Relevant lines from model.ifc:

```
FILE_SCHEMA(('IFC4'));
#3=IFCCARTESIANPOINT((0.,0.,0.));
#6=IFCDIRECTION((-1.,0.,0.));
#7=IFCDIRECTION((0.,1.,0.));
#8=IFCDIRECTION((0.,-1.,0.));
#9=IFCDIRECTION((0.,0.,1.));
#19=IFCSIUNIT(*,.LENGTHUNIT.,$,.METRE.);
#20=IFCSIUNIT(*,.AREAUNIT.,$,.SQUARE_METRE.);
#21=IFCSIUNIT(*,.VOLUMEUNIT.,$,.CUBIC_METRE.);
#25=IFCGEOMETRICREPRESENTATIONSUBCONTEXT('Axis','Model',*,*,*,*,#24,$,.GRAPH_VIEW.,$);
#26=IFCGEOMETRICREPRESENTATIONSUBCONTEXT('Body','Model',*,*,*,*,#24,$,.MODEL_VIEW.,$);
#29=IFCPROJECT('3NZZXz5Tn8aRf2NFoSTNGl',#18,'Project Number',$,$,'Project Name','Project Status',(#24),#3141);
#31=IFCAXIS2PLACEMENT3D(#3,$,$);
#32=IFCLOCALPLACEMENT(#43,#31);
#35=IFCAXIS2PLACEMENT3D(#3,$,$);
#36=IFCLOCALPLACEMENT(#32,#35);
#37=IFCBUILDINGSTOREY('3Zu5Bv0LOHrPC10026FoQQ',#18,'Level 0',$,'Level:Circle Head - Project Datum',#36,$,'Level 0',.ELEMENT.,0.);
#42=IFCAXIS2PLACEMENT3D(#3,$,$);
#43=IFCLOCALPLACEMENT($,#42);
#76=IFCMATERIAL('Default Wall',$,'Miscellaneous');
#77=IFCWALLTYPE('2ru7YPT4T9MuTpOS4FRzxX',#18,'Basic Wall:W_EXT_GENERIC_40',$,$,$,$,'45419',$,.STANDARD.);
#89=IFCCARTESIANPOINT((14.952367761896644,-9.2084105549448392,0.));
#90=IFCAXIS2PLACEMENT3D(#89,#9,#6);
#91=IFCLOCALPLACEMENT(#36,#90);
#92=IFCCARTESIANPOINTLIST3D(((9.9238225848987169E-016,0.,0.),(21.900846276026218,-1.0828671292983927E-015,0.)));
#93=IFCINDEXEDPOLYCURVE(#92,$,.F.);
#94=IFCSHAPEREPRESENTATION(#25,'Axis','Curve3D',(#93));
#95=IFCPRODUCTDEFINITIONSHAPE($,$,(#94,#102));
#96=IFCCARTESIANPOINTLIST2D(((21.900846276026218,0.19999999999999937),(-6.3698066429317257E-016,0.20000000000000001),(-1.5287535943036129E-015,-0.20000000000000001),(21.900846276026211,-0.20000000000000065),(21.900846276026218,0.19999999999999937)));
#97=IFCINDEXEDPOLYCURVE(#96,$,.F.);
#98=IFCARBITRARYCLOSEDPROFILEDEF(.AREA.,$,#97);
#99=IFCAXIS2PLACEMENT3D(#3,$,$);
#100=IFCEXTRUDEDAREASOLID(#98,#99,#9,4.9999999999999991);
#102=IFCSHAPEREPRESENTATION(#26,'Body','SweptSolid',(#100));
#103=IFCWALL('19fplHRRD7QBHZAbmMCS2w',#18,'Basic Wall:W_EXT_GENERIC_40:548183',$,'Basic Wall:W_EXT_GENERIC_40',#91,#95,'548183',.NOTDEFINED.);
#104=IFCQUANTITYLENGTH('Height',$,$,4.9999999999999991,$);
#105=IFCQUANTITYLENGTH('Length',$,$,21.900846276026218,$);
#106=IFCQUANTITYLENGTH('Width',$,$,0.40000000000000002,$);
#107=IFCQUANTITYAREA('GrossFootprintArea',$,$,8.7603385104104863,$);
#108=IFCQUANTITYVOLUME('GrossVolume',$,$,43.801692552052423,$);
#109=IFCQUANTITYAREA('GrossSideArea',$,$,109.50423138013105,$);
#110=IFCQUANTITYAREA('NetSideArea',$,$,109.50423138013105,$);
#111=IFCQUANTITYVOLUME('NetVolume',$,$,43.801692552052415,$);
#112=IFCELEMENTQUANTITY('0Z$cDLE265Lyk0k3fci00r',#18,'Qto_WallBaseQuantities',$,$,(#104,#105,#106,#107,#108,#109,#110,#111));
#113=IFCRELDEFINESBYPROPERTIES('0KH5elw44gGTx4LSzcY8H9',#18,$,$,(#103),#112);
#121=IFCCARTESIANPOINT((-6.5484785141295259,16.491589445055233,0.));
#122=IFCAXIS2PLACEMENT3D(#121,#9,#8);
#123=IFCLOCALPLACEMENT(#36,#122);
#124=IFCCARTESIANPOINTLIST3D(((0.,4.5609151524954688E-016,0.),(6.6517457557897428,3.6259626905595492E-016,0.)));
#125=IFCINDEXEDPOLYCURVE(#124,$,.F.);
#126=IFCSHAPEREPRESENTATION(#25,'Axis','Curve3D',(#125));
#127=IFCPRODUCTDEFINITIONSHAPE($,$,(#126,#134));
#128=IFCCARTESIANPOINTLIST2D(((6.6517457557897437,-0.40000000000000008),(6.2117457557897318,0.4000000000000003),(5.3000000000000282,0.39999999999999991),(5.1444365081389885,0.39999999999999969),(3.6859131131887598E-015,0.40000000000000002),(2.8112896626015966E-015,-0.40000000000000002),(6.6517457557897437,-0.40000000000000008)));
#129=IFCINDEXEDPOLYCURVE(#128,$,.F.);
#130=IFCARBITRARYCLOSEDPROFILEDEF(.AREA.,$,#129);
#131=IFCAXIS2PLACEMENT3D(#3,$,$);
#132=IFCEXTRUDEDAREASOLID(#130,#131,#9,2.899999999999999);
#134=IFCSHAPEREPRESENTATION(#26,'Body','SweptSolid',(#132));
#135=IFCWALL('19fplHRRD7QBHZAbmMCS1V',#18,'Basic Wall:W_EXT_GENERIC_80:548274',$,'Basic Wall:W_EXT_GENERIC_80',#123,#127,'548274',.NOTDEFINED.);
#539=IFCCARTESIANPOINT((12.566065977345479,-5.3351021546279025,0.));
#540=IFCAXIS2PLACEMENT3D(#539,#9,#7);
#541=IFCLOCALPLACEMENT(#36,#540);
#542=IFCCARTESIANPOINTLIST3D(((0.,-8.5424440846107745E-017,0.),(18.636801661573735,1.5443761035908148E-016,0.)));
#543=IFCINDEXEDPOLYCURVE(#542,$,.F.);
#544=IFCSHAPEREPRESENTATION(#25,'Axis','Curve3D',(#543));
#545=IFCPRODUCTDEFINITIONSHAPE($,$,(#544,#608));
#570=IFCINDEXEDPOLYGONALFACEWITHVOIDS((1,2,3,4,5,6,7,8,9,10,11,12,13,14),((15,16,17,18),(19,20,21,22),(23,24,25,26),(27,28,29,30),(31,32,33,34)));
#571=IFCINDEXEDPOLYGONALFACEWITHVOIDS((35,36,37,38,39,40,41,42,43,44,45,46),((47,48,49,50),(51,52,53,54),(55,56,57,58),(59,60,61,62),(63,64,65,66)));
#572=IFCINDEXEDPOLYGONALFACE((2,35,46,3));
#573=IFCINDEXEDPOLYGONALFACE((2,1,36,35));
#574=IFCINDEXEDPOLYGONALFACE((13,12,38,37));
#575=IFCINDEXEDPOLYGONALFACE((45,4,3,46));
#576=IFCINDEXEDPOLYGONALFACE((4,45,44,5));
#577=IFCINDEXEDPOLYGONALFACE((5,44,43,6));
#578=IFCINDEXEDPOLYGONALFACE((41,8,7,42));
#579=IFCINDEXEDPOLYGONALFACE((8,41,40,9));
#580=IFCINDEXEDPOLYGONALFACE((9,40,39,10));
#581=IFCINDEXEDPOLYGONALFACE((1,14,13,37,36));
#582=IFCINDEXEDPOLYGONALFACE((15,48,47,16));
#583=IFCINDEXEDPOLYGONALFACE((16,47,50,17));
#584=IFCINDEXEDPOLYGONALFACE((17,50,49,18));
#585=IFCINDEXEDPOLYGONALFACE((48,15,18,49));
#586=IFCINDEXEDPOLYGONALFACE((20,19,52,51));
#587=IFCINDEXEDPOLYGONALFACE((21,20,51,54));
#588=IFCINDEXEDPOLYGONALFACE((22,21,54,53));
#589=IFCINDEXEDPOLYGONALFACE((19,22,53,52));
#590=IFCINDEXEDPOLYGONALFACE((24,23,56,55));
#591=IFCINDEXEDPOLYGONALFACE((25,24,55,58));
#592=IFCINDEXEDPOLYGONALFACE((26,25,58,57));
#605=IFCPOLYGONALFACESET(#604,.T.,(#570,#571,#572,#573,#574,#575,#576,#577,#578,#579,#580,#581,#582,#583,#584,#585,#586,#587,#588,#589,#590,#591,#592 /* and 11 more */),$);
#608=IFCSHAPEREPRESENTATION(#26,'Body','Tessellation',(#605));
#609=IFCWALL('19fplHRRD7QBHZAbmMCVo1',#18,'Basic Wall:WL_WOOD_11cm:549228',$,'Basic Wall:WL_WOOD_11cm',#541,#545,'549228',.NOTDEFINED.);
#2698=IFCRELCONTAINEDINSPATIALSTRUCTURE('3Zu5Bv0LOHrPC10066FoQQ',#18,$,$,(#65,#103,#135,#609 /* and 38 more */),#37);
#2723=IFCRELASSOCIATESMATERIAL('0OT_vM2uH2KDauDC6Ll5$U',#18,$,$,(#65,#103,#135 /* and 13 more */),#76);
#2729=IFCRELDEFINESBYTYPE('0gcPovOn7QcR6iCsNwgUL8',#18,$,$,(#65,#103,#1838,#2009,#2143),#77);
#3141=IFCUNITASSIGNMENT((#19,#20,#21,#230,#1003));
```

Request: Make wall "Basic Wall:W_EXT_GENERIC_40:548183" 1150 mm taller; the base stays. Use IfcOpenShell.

```python
import ifcopenshell
import ifcopenshell.api.pset
import ifcopenshell.geom
import ifcopenshell.util.element
import ifcopenshell.util.representation
import ifcopenshell.util.shape
import ifcopenshell.util.unit

model = ifcopenshell.open("model.ifc")
unit_scale = ifcopenshell.util.unit.calculate_unit_scale(model)
area_scale = ifcopenshell.util.unit.calculate_unit_scale(model, "AREAUNIT")
volume_scale = ifcopenshell.util.unit.calculate_unit_scale(model, "VOLUMEUNIT")
settings = ifcopenshell.geom.settings()


def volume(element):
    """Net volume in cubic metres, openings subtracted."""
    shape = ifcopenshell.geom.create_shape(settings, element)
    return ifcopenshell.util.shape.get_volume(shape.geometry)


wall = model.by_guid("19fplHRRD7QBHZAbmMCS2w")
before = volume(wall)

body = ifcopenshell.util.representation.get_representation(wall, "Model", "Body")
solid = body.Items[0]
old_height = solid.Depth
solid.Depth += 1.15
after = volume(wall)
thickness = 0.4  # wall thickness in metres

# Update the stored height, areas and volumes.
qto = model.by_id(ifcopenshell.util.element.get_pset(wall, "Qto_WallBaseQuantities", should_inherit=False)["id"])
ifcopenshell.api.pset.edit_qto(model, qto=qto, properties={
    "Height": solid.Depth,
    "GrossVolume": ifcopenshell.util.element.get_pset(wall, "Qto_WallBaseQuantities", "GrossVolume") * solid.Depth / old_height,
    "GrossSideArea": ifcopenshell.util.element.get_pset(wall, "Qto_WallBaseQuantities", "GrossSideArea") * solid.Depth / old_height,
    "NetSideArea": after / thickness / area_scale,
    "NetVolume": after / volume_scale,
})

print(f"height {old_height:g} -> {solid.Depth:g}, volume {before:.3f} -> {after:.3f} m3")

model.write("model_v2.ifc")
```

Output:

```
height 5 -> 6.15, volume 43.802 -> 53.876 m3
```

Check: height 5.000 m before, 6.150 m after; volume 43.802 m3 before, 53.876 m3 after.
